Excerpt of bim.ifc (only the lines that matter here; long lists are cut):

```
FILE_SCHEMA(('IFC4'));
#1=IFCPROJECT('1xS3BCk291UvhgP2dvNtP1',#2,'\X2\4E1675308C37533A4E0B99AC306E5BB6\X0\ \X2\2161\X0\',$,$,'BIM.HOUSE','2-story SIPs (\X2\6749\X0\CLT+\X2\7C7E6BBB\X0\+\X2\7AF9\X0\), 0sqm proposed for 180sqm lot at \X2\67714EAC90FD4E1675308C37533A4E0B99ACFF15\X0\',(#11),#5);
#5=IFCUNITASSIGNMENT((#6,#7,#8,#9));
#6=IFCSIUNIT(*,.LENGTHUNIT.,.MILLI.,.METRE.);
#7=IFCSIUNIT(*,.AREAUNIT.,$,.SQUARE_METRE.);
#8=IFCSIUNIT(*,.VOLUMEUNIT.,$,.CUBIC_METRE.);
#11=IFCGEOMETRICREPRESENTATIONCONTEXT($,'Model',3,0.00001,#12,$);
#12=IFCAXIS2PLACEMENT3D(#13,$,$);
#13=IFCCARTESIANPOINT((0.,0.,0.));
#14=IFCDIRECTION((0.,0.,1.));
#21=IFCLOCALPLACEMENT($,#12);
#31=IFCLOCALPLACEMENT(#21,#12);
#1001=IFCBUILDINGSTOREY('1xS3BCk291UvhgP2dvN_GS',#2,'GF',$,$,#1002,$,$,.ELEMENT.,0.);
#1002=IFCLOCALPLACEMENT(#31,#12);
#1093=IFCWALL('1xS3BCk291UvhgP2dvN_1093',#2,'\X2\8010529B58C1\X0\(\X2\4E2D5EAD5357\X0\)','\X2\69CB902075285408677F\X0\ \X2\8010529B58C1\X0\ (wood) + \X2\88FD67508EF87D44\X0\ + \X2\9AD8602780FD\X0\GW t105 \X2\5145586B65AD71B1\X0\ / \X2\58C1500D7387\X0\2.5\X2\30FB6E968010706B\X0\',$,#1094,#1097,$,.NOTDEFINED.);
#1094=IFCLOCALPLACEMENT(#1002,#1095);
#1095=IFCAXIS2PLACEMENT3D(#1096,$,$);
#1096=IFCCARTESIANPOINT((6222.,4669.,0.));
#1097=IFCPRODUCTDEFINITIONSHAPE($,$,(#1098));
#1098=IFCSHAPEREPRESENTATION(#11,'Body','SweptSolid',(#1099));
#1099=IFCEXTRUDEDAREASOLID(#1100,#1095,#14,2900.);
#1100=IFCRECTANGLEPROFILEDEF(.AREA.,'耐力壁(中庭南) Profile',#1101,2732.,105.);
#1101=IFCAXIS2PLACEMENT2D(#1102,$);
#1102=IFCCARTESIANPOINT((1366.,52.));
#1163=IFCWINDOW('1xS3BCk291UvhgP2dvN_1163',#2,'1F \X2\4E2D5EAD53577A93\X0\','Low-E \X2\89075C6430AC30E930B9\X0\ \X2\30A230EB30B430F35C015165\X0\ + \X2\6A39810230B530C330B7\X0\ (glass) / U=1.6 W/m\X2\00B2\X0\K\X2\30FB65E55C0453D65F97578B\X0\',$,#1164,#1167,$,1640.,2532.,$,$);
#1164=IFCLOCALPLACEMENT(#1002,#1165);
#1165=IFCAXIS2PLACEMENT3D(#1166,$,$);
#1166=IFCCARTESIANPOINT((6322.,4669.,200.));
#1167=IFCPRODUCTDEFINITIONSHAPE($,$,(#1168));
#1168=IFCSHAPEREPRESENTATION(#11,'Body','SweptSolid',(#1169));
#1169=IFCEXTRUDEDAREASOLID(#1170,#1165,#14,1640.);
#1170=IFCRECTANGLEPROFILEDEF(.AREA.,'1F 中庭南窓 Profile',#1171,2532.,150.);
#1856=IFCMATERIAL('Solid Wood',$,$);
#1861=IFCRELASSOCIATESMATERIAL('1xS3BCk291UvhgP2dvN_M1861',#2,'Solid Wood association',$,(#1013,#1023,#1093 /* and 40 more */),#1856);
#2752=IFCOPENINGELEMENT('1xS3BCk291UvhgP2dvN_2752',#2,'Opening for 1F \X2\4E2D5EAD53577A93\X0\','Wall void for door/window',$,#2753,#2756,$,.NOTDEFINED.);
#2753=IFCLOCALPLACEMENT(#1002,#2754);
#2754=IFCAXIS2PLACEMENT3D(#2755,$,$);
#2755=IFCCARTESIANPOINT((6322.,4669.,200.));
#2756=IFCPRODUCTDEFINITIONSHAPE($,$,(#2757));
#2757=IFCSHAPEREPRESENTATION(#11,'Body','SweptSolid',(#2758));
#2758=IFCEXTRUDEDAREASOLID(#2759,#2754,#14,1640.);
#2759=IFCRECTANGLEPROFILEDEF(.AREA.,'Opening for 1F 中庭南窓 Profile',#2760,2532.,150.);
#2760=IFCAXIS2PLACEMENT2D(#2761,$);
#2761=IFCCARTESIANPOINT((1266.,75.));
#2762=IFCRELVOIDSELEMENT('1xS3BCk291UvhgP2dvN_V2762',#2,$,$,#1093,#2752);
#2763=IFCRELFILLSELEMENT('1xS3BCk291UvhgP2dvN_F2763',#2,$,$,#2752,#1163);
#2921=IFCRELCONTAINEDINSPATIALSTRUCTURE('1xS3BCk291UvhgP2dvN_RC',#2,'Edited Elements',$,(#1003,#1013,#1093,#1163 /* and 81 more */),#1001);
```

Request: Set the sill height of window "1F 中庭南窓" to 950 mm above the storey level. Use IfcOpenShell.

```python
import numpy as np
import ifcopenshell
import ifcopenshell.api.geometry
import ifcopenshell.geom
import ifcopenshell.util.element
import ifcopenshell.util.placement
import ifcopenshell.util.shape
import ifcopenshell.util.unit

model = ifcopenshell.open("bim.ifc")
unit_scale = ifcopenshell.util.unit.calculate_unit_scale(model)

window = model.by_id(1163)
opening = window.FillsVoids[0].RelatingOpeningElement
storey = ifcopenshell.util.element.get_container(window, ifc_class="IfcBuildingStorey")
level = ifcopenshell.util.placement.get_local_placement(storey.ObjectPlacement)[2, 3]

# The opening's origin need not be at the sill, so measure its lowest point.
shape = ifcopenshell.geom.create_shape(ifcopenshell.geom.settings(), opening)
bottom = ifcopenshell.util.shape.get_shape_bottom_elevation(shape, shape.geometry) / unit_scale
dz = level + 0.95 / unit_scale - bottom

shift = np.array([0.0, 0.0, dz])
# The window is not placed relative to its opening, so move both.
for product in (opening, window):
    matrix = ifcopenshell.util.placement.get_local_placement(product.ObjectPlacement)
    matrix[:3, 3] += shift
    ifcopenshell.api.geometry.edit_object_placement(model, product=product, matrix=matrix, is_si=False)

print(f"moved by {dz * unit_scale:+.3f} m")

model.write("bim_v2.ifc")
```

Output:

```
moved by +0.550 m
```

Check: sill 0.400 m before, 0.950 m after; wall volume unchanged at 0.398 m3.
